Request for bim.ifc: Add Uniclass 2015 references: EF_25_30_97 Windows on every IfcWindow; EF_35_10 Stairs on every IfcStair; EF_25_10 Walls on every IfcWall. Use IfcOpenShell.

First a look at what the model holds.

```python
import ifcopenshell

model = ifcopenshell.open("bim.ifc")
print(model.schema)
print("classifications:", [c.Name for c in model.by_type("IfcClassification")])
for ifc_class in ("IfcDoor", "IfcRoof", "IfcStair", "IfcWall", "IfcWindow"):
    print(ifc_class, len(model.by_type(ifc_class)))
```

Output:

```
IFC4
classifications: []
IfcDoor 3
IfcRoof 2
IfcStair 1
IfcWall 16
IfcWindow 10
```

```python
import ifcopenshell
import ifcopenshell.api.classification

model = ifcopenshell.open("bim.ifc")

system = ifcopenshell.api.classification.add_classification(model, classification="Uniclass 2015")

codes = {
    "IfcWindow": ("EF_25_30_97", "Windows"),
    "IfcStair": ("EF_35_10", "Stairs"),
    "IfcWall": ("EF_25_10", "Walls"),
}
for ifc_class, (code, name) in codes.items():
    products = model.by_type(ifc_class)
    ifcopenshell.api.classification.add_reference(
        model, products=products, classification=system, identification=code, name=name
    )
    print(code, len(products))

model.write("bim-out.ifc")
```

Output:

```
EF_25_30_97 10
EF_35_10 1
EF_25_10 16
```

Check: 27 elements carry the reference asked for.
